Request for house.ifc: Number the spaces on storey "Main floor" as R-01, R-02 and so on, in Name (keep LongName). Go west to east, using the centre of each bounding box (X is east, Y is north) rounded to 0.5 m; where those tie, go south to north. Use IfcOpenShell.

First a look at what the model holds.

```python
import ifcopenshell
import ifcopenshell.util.element
import ifcopenshell.util.placement

model = ifcopenshell.open("house.ifc")
print(model.schema)
storey = next(s for s in model.by_type("IfcBuildingStorey") if s.Name == "Main floor")
spaces = [e for e in ifcopenshell.util.element.get_decomposition(storey) if e.is_a("IfcSpace")]
for e in sorted(spaces, key=lambda e: e.id()):
    origin = ifcopenshell.util.placement.get_local_placement(e.ObjectPlacement)[:3, 3]
    print(e.id(), e.Name, e.LongName, origin.round(2) + 0.0, sep=" | ")
```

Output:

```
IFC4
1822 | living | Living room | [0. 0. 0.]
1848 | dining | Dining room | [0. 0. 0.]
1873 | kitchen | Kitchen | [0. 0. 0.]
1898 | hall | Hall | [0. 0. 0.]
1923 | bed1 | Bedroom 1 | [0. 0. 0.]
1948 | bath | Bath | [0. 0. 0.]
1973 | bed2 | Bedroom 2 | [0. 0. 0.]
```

```python
import ifcopenshell
import ifcopenshell.geom
import ifcopenshell.util.element
import ifcopenshell.util.shape

model = ifcopenshell.open("house.ifc")
settings = ifcopenshell.geom.settings()
settings.set("use-world-coords", True)


def centre(element):
    shape = ifcopenshell.geom.create_shape(settings, element)
    return ifcopenshell.util.shape.get_bbox_centroid(shape.geometry)


storey = next(s for s in model.by_type("IfcBuildingStorey") if s.Name == "Main floor")
spaces = [e for e in ifcopenshell.util.element.get_decomposition(storey) if e.is_a("IfcSpace")]

# Insertion points can sit at a corner or the storey origin, so sort by the geometry (in metres).
centres = {e: centre(e) for e in spaces}
spaces.sort(key=lambda e: (round(centres[e][0] / 0.5), centres[e][1]))

for i, e in enumerate(spaces, start=1):
    number = f"R-{i:02d}"
    e.Name = number
    print(e.id(), number)

model.write("house_v2.ifc")
```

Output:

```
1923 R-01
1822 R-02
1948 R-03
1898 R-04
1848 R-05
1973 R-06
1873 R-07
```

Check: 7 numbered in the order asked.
